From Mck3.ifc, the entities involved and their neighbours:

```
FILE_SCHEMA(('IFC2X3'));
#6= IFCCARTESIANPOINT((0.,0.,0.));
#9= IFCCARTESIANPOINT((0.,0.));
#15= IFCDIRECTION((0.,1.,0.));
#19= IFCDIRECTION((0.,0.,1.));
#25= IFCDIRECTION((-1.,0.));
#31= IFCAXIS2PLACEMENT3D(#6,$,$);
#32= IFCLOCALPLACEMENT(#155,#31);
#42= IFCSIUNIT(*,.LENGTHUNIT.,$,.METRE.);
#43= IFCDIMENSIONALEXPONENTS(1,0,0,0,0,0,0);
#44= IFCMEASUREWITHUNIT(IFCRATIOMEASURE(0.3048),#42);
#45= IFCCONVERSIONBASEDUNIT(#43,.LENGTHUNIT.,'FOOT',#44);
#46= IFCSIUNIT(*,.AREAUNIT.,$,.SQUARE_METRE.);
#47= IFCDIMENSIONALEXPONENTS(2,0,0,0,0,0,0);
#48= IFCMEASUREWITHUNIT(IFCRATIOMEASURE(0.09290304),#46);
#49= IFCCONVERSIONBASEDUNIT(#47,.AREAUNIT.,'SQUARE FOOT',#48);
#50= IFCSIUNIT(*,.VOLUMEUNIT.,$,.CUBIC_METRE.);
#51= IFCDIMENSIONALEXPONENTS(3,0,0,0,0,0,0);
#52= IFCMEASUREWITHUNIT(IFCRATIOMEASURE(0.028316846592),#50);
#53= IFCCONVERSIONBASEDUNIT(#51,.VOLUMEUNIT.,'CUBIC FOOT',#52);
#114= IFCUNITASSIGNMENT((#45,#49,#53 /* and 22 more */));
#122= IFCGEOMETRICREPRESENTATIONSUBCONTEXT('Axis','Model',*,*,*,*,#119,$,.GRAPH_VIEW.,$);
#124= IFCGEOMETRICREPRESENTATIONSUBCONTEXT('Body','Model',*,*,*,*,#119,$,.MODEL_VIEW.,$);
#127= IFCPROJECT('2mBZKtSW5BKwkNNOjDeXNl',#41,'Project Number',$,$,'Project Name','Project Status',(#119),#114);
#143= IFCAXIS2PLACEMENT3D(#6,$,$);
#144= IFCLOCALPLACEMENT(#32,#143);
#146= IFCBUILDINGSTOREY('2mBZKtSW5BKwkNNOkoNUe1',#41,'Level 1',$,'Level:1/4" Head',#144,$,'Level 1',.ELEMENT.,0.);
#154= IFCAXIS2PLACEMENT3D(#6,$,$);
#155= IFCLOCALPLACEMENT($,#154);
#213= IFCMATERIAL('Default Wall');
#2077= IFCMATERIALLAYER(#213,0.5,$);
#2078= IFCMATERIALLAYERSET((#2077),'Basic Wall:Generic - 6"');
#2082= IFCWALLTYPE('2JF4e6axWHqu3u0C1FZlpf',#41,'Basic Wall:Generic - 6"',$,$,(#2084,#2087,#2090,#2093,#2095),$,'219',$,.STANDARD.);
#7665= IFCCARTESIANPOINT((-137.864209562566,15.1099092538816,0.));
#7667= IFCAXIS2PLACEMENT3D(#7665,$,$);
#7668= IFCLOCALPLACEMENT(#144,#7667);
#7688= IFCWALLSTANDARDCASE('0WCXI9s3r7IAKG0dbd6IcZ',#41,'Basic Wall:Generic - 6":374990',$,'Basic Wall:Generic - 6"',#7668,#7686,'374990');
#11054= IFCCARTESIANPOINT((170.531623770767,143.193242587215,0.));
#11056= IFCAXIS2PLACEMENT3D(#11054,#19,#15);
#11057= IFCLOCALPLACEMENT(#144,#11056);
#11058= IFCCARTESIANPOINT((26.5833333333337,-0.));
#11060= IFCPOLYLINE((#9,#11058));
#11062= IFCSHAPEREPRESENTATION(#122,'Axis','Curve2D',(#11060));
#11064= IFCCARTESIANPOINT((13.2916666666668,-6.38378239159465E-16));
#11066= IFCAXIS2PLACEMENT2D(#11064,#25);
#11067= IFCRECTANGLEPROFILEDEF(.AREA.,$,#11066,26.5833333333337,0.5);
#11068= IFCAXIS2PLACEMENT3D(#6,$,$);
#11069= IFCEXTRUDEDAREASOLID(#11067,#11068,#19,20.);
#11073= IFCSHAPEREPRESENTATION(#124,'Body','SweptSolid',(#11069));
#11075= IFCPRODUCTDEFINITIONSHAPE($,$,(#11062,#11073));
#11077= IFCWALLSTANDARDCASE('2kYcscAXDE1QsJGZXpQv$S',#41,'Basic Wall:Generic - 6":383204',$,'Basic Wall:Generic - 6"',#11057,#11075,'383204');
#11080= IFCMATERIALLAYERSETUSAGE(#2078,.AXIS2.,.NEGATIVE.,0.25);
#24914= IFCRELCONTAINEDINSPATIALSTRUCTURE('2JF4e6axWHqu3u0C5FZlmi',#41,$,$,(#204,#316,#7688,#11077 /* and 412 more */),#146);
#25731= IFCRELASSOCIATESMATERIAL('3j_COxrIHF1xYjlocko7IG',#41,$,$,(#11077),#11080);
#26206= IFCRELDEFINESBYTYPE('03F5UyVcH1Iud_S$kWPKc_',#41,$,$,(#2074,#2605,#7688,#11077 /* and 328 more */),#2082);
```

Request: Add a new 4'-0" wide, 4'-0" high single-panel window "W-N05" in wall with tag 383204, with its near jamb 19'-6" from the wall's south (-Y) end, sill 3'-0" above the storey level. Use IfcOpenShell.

```python
import numpy as np
import ifcopenshell
import ifcopenshell.api.feature
import ifcopenshell.api.geometry
import ifcopenshell.api.root
import ifcopenshell.api.spatial
import ifcopenshell.api.type
import ifcopenshell.geom
import ifcopenshell.util.element
import ifcopenshell.util.placement
import ifcopenshell.util.representation
import ifcopenshell.util.shape
import ifcopenshell.util.unit

model = ifcopenshell.open("Mck3.ifc")
unit_scale = ifcopenshell.util.unit.calculate_unit_scale(model)
settings = ifcopenshell.geom.settings()


def volume(element):
    """Net volume in cubic metres, openings subtracted."""
    shape = ifcopenshell.geom.create_shape(settings, element)
    return ifcopenshell.util.shape.get_volume(shape.geometry)


wall = model.by_id(11077)
storey = ifcopenshell.util.element.get_container(wall, ifc_class="IfcBuildingStorey")
context = ifcopenshell.util.representation.get_context(model, "Model", "Body", "MODEL_VIEW")
before = volume(wall)

width, height, from_end, sill = 1.2192, 1.2192, 5.9436, 0.9144  # metres

# The wall runs along its own X axis, and the end named is its -X end.
wall_shape = ifcopenshell.geom.create_shape(settings, wall)
x, y, z = ifcopenshell.util.shape.get_vertices(wall_shape.geometry).T
start = x.min() + from_end
face, thickness = float(y.min()), float(y.max() - y.min())
wall_matrix = ifcopenshell.util.placement.get_local_placement(wall.ObjectPlacement)
level = ifcopenshell.util.placement.get_local_placement(storey.ObjectPlacement)[2, 3]


def in_wall(x, y):
    """Placement at x, y metres in the wall's axes, at sill height."""
    matrix = wall_matrix.copy()
    matrix[:, 3] = wall_matrix @ np.array([x / unit_scale, y / unit_scale, 0.0, 1.0])
    matrix[2, 3] = level + sill / unit_scale
    return matrix


# Opening: a box that overshoots both wall faces by 50 mm.
opening = ifcopenshell.api.root.create_entity(model, ifc_class="IfcOpeningElement")
box = ifcopenshell.api.geometry.add_wall_representation(
    model, context=context, length=width, height=height, thickness=thickness + 0.1
)
ifcopenshell.api.geometry.assign_representation(model, product=opening, representation=box)
ifcopenshell.api.geometry.edit_object_placement(model, product=opening, matrix=in_wall(start, face - 0.05), is_si=False)
ifcopenshell.api.feature.add_feature(model, feature=opening, element=wall)

window = ifcopenshell.api.root.create_entity(model, ifc_class="IfcWindow", name="W-N05")
window.OverallWidth, window.OverallHeight = width / unit_scale, height / unit_scale
body = ifcopenshell.api.geometry.add_window_representation(
    model,
    context=context,
    overall_width=window.OverallWidth,
    overall_height=window.OverallHeight,
    partition_type="SINGLE_PANEL",
)
ifcopenshell.api.geometry.assign_representation(model, product=window, representation=body)
ifcopenshell.api.spatial.assign_container(model, products=[window], relating_structure=storey)
fills = ifcopenshell.api.feature.add_filling(model, opening=opening, element=window)
fills.OwnerHistory = window.OwnerHistory  # required in IFC2X3

# IFC2X3 keeps the operation on the window style.
style = ifcopenshell.api.root.create_entity(model, ifc_class="IfcWindowStyle", name="W-N05")
style.OperationType, style.ConstructionType = "SINGLE_PANEL", "NOTDEFINED"
style.ParameterTakesPrecedence = style.Sizeable = False
ifcopenshell.api.type.assign_type(model, related_objects=[window], relating_type=style)

# Centre the window in the wall's thickness.
ifcopenshell.api.geometry.edit_object_placement(model, product=window, matrix=in_wall(start, face), is_si=False)
window_shape = ifcopenshell.geom.create_shape(settings, window)
depth = ifcopenshell.util.shape.get_vertices(window_shape.geometry)[:, 1]
offset = face + thickness / 2 - (depth.min() + depth.max()) / 2
ifcopenshell.api.geometry.edit_object_placement(model, product=window, matrix=in_wall(start, offset), is_si=False)

after = volume(wall)

print(f"wall volume {before:.3f} -> {after:.3f} m3")

model.write("Mck3_v2.ifc")
```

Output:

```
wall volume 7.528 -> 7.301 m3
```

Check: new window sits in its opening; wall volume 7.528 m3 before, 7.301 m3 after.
